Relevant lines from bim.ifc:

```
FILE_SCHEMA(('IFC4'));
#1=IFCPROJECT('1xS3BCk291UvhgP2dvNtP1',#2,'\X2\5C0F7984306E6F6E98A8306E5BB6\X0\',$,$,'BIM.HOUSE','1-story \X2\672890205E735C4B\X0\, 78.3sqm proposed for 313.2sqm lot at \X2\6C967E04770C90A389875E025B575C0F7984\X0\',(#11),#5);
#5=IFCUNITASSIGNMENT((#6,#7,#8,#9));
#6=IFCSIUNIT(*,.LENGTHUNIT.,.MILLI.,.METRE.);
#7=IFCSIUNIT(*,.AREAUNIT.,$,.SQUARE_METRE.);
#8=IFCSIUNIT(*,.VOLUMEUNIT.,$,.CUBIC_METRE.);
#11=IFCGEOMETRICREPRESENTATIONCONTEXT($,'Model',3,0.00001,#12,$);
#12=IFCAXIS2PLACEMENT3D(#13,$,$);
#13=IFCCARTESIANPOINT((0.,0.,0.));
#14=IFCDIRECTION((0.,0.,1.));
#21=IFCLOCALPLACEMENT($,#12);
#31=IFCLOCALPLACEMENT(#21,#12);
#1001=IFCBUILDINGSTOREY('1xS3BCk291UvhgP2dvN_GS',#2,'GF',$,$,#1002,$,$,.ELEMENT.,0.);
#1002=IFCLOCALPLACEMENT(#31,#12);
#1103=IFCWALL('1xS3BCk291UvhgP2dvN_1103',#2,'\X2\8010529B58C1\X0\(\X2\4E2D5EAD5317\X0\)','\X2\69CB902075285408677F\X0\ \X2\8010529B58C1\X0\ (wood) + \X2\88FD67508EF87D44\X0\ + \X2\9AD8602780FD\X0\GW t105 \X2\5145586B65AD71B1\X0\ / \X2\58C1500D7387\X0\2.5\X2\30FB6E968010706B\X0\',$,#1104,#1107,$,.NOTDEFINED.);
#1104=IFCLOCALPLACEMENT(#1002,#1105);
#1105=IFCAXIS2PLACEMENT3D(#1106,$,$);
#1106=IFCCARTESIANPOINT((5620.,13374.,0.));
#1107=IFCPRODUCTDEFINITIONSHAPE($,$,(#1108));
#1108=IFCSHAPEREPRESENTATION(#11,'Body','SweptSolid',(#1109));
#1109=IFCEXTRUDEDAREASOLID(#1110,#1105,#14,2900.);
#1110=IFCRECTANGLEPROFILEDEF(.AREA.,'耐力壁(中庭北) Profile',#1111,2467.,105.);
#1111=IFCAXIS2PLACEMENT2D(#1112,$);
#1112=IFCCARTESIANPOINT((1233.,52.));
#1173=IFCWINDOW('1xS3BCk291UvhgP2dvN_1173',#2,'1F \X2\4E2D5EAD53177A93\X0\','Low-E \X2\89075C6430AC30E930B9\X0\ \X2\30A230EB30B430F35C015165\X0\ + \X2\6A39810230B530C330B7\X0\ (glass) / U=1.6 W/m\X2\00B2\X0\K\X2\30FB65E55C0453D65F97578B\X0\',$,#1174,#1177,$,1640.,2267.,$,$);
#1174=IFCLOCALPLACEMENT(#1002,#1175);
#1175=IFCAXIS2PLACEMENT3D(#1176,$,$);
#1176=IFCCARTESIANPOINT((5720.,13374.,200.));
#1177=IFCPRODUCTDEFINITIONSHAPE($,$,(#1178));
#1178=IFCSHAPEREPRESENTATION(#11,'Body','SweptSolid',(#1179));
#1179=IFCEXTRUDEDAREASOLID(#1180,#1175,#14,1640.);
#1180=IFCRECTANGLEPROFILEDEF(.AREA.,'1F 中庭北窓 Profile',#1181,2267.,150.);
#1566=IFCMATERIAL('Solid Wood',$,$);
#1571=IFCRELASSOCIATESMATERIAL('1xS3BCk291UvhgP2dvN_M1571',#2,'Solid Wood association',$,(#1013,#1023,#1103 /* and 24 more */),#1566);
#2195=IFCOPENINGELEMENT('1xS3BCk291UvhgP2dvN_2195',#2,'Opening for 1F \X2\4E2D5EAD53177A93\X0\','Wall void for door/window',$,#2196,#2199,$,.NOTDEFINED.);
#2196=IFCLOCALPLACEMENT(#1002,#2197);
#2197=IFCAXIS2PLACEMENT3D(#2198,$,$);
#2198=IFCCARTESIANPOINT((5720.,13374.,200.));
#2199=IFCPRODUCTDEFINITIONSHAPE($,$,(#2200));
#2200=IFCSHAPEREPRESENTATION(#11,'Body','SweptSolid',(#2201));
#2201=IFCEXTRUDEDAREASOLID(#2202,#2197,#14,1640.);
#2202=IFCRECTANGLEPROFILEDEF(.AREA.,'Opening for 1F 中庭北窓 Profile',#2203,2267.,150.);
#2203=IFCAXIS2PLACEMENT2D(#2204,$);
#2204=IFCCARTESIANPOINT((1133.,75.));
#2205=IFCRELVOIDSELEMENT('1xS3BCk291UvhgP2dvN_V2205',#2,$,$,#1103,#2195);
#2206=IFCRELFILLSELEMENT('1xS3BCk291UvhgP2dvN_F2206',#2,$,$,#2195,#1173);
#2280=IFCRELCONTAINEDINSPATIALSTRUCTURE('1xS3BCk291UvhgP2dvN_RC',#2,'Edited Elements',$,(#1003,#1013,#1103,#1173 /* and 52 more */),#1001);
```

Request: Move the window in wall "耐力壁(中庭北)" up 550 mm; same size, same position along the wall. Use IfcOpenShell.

```python
import numpy as np
import ifcopenshell
import ifcopenshell.api.geometry
import ifcopenshell.util.placement
import ifcopenshell.util.unit

model = ifcopenshell.open("bim.ifc")
unit_scale = ifcopenshell.util.unit.calculate_unit_scale(model)

window = model.by_guid("1xS3BCk291UvhgP2dvN_1173")
opening = window.FillsVoids[0].RelatingOpeningElement
dz = 0.55 / unit_scale

shift = np.array([0.0, 0.0, dz])
# The window is not placed relative to its opening, so move both.
for product in (opening, window):
    matrix = ifcopenshell.util.placement.get_local_placement(product.ObjectPlacement)
    matrix[:3, 3] += shift
    ifcopenshell.api.geometry.edit_object_placement(model, product=product, matrix=matrix, is_si=False)

print(f"moved by {dz * unit_scale:+.3f} m")

model.write("bim_updated.ifc")
```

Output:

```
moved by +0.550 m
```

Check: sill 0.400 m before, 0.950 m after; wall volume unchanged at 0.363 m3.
